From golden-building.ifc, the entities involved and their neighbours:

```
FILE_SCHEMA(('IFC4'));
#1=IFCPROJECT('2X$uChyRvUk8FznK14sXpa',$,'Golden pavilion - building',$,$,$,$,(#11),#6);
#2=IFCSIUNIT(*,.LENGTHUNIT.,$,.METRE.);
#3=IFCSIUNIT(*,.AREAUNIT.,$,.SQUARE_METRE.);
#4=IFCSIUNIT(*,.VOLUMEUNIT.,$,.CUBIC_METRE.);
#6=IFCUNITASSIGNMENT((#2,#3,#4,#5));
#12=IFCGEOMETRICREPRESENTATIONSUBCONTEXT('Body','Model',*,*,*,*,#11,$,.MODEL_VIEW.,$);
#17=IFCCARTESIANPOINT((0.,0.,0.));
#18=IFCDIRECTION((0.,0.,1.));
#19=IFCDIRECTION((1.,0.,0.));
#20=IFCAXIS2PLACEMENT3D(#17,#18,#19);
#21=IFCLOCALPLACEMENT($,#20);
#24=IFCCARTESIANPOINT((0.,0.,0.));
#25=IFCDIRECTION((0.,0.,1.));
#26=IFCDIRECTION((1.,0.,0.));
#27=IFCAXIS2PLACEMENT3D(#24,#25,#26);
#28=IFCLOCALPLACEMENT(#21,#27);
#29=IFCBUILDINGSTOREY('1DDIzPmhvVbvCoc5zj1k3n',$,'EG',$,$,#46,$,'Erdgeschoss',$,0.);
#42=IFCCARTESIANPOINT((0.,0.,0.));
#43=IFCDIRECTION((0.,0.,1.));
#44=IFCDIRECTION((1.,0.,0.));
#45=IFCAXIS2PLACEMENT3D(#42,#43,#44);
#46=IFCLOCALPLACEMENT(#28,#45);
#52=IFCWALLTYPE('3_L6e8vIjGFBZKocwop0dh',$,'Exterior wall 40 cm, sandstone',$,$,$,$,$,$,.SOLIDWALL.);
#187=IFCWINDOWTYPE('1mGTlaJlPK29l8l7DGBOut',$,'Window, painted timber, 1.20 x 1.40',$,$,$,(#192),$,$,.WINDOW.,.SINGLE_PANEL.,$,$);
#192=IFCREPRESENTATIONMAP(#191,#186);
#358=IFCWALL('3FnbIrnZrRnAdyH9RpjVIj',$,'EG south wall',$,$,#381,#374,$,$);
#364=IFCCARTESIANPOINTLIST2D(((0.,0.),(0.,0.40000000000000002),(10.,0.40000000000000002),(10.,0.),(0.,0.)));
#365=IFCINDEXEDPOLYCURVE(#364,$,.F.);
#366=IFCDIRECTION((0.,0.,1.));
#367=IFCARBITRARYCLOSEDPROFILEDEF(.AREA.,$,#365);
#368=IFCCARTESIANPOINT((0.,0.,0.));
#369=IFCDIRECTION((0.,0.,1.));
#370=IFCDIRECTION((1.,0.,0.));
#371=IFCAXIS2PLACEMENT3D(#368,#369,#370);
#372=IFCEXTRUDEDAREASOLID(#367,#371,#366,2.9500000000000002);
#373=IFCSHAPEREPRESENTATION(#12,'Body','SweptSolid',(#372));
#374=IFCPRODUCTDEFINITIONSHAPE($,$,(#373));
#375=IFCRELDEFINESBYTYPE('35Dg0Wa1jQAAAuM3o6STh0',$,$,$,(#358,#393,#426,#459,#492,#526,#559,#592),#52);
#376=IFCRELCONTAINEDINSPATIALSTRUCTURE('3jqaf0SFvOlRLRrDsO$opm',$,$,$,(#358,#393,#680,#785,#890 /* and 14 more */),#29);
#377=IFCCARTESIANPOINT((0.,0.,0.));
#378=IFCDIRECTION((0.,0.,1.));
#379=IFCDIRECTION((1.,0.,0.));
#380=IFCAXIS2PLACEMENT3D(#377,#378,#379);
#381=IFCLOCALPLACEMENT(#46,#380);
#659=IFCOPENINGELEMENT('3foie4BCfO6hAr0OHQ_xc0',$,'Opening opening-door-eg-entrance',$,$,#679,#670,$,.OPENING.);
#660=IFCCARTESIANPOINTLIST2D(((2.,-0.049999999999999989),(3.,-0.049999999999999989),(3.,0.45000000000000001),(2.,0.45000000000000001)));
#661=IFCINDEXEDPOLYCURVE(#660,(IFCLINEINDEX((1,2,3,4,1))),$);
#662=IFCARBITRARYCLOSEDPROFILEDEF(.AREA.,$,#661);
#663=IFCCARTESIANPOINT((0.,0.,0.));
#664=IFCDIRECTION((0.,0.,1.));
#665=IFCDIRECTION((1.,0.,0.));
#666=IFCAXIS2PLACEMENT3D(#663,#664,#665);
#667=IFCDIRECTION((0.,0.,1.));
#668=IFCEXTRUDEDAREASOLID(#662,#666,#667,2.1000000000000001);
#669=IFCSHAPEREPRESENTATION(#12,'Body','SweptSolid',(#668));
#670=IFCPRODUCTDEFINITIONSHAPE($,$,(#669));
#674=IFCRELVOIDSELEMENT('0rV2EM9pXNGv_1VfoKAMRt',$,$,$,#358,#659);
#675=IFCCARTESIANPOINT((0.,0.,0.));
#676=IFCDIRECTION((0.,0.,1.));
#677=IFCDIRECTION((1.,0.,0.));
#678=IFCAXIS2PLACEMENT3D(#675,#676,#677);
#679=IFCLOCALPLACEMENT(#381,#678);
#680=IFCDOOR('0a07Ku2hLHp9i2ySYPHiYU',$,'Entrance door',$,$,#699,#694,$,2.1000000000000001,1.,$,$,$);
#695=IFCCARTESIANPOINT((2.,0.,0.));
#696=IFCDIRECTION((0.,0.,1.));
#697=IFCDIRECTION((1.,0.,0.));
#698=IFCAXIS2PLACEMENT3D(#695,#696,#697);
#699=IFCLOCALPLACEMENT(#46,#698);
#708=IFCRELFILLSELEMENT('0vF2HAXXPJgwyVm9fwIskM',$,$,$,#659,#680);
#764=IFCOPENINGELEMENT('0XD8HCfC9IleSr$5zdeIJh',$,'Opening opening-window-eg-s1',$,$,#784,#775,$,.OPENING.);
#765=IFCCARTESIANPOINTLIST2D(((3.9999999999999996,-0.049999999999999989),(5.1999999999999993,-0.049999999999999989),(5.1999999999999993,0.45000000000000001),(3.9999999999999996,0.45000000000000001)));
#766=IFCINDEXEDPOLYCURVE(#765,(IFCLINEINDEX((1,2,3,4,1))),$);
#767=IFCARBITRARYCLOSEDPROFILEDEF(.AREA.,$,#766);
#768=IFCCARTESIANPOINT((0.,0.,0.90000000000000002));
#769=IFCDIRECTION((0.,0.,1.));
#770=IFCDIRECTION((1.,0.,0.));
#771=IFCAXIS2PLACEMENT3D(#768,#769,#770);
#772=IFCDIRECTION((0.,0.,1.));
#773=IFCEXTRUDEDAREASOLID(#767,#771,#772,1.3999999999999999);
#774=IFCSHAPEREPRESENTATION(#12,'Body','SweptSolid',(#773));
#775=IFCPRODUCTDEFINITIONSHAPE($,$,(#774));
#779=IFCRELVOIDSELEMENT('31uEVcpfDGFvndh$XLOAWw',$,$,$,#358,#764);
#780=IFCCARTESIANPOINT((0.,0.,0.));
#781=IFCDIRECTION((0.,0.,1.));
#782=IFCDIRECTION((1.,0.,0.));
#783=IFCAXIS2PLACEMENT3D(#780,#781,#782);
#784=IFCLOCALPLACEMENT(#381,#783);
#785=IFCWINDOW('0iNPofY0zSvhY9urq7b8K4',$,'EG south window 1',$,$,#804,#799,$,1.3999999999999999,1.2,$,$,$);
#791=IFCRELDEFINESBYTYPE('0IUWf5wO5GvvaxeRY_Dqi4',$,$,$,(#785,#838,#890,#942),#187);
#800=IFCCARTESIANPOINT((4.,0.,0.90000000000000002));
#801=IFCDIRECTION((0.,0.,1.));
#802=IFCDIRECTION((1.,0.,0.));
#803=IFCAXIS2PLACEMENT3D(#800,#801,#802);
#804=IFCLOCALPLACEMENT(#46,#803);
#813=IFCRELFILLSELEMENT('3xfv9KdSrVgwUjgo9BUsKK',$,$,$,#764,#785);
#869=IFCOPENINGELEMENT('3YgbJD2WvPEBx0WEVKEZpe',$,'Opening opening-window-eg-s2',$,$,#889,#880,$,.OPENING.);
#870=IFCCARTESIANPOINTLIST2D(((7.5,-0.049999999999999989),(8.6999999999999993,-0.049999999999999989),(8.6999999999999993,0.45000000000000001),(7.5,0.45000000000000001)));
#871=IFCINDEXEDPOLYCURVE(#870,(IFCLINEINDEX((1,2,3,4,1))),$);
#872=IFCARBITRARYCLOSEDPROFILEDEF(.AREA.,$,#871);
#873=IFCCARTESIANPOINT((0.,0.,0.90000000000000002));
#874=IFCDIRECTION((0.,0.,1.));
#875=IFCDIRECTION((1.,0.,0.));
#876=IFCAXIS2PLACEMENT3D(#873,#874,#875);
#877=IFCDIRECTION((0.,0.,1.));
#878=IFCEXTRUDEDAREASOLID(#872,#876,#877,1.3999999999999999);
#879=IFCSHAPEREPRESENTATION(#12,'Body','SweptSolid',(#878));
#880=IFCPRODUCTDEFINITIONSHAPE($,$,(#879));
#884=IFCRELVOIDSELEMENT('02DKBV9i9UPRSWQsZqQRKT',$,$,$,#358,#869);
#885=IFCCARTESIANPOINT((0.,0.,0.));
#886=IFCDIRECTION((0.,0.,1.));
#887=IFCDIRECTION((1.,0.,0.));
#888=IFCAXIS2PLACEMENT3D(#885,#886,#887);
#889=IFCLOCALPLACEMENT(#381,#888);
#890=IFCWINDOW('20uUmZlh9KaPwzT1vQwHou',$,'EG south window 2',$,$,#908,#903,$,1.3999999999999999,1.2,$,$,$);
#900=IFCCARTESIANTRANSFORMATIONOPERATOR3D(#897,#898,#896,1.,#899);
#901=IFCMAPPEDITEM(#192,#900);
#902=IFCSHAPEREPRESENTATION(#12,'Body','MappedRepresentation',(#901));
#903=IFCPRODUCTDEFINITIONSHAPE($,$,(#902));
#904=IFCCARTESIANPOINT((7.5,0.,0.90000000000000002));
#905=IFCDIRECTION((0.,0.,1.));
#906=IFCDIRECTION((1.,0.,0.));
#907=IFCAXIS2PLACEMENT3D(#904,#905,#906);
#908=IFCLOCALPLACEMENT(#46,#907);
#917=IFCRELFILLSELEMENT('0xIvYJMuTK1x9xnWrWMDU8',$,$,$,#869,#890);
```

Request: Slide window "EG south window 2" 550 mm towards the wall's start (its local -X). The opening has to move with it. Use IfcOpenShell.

```python
import ifcopenshell
import ifcopenshell.api.geometry
import ifcopenshell.util.placement
import ifcopenshell.util.unit

model = ifcopenshell.open("golden-building.ifc")
unit_scale = ifcopenshell.util.unit.calculate_unit_scale(model)

window = model.by_guid("20uUmZlh9KaPwzT1vQwHou")
opening = window.FillsVoids[0].RelatingOpeningElement
wall = opening.VoidsElements[0].RelatingBuildingElement

wall_matrix = ifcopenshell.util.placement.get_local_placement(wall.ObjectPlacement)
shift = wall_matrix[:3, 0] * -0.55 / unit_scale
before = ifcopenshell.util.placement.get_local_placement(window.ObjectPlacement)[:3, 3].copy()

# The window is not placed relative to its opening, so move both.
for product in (opening, window):
    matrix = ifcopenshell.util.placement.get_local_placement(product.ObjectPlacement)
    matrix[:3, 3] += shift
    ifcopenshell.api.geometry.edit_object_placement(model, product=product, matrix=matrix, is_si=False)

after = ifcopenshell.util.placement.get_local_placement(window.ObjectPlacement)[:3, 3]
print("window moved by", (after - before).round(3) + 0.0)

model.write("golden-building_v2.ifc")
```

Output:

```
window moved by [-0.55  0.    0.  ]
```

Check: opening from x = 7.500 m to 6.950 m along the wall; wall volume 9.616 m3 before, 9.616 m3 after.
